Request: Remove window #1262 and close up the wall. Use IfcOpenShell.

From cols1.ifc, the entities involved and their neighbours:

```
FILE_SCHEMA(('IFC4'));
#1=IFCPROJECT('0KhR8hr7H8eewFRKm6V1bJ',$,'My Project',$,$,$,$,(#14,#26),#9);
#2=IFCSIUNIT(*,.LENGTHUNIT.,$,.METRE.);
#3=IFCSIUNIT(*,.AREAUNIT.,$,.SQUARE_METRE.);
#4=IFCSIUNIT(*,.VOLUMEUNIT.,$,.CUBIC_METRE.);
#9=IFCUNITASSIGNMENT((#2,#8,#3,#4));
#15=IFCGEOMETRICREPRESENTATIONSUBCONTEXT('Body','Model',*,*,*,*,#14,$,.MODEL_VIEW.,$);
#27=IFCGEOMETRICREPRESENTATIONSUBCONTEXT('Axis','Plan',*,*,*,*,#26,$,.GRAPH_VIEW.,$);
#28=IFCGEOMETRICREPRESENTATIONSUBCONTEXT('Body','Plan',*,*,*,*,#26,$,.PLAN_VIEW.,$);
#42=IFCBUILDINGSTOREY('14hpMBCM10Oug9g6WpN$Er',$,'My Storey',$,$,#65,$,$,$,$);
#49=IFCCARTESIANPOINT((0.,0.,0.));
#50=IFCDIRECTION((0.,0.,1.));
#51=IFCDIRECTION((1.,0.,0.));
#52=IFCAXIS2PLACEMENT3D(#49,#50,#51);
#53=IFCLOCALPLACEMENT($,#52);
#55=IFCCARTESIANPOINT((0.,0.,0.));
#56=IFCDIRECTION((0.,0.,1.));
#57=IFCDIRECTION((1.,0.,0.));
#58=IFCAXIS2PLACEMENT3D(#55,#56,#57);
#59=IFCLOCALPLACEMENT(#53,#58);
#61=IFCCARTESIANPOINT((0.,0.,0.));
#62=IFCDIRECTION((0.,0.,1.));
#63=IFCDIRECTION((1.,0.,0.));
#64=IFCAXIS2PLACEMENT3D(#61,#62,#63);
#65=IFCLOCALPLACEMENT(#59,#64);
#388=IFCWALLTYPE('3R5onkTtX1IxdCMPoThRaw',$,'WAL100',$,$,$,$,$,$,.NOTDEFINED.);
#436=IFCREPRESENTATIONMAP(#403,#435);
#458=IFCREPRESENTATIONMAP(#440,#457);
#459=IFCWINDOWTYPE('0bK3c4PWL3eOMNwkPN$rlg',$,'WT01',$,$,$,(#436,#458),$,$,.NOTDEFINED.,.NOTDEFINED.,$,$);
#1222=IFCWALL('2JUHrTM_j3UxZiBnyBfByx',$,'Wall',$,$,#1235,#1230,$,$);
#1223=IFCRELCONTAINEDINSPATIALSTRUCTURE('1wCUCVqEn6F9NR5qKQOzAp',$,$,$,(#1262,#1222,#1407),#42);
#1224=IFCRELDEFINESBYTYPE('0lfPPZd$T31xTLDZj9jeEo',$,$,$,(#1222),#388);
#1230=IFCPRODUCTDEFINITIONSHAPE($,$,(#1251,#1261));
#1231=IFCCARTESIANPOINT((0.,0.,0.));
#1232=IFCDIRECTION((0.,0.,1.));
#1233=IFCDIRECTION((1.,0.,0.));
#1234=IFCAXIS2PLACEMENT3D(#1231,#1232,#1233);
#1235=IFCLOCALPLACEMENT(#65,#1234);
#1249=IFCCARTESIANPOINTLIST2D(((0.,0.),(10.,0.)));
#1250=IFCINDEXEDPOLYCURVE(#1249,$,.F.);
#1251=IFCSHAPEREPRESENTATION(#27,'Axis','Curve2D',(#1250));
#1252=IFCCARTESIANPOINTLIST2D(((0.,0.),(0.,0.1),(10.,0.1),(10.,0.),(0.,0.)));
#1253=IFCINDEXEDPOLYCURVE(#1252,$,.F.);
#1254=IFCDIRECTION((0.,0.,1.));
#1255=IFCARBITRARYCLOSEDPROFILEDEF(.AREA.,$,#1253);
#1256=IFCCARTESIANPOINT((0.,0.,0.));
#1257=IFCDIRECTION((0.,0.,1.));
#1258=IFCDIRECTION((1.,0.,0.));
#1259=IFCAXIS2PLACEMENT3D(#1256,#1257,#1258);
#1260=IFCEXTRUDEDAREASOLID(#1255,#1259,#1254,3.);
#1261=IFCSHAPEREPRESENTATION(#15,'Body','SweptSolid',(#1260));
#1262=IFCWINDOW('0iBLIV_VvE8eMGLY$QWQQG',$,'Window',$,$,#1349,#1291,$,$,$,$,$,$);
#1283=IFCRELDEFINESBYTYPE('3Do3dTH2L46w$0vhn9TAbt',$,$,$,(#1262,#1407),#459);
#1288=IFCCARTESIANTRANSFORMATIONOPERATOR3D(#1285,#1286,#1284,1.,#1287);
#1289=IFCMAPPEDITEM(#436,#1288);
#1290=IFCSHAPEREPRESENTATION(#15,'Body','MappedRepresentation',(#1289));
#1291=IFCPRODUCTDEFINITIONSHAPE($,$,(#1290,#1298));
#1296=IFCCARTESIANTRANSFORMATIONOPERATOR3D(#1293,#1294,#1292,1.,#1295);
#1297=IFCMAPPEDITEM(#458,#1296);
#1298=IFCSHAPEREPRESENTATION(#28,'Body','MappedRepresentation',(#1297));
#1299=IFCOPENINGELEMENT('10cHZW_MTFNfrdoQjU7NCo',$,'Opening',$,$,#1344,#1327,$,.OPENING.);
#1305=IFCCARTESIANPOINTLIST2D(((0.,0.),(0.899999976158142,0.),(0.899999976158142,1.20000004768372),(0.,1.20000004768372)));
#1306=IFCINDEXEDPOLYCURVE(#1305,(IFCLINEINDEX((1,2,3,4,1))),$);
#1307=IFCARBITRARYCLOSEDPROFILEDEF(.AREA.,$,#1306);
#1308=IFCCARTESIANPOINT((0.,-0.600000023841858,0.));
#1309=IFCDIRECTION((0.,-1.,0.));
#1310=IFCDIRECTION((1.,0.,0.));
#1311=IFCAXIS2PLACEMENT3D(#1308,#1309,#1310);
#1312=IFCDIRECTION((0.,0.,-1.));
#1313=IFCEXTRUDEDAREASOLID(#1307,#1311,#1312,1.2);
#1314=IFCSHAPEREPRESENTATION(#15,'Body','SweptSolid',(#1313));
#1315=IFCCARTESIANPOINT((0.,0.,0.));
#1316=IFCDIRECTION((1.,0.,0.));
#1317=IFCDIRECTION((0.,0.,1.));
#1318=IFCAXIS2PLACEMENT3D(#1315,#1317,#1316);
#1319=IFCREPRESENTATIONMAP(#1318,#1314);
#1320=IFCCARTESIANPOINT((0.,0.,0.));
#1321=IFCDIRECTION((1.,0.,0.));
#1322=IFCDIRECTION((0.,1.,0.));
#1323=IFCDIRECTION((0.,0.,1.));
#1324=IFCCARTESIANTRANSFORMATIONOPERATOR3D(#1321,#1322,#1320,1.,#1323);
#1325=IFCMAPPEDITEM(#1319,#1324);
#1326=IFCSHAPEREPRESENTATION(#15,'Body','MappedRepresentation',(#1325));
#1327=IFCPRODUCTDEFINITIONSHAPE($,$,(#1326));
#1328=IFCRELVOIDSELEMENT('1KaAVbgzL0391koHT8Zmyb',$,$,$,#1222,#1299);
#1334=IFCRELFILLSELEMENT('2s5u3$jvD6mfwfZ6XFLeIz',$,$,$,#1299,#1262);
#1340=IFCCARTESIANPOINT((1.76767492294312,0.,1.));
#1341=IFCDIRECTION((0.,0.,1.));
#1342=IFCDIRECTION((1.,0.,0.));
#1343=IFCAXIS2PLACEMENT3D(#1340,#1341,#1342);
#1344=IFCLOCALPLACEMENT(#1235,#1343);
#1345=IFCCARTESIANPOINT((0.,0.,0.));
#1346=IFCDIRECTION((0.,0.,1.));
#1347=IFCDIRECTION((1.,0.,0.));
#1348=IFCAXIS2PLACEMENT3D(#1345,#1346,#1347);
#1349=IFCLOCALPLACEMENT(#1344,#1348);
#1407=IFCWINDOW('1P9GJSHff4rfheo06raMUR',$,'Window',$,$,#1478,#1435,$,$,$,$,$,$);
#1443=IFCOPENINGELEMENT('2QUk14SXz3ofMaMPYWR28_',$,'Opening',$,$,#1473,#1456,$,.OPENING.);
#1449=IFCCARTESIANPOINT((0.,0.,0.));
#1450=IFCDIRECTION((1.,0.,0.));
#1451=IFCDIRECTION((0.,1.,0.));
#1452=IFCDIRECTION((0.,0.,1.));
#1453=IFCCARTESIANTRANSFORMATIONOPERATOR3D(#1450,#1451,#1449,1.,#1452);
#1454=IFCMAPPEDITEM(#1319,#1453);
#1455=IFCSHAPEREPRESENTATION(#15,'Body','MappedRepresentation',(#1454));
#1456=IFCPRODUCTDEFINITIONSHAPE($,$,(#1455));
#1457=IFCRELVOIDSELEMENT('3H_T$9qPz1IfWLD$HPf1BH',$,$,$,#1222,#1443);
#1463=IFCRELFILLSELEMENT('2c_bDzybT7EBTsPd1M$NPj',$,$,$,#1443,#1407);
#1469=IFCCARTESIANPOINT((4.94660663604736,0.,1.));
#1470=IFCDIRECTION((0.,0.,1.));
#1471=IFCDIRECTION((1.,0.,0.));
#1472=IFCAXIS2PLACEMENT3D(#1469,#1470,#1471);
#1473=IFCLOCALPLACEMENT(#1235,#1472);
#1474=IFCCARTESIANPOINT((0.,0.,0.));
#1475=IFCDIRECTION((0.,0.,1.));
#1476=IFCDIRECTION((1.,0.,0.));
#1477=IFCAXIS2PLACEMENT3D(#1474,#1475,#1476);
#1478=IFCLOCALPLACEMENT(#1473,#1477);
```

```python
import ifcopenshell
import ifcopenshell.api.feature
import ifcopenshell.api.root
import ifcopenshell.geom
import ifcopenshell.util.shape

model = ifcopenshell.open("cols1.ifc")
settings = ifcopenshell.geom.settings()


def volume(element):
    """Net volume in cubic metres, openings subtracted."""
    shape = ifcopenshell.geom.create_shape(settings, element)
    return ifcopenshell.util.shape.get_volume(shape.geometry)


window = model.by_guid("0iBLIV_VvE8eMGLY$QWQQG")
opening = window.FillsVoids[0].RelatingOpeningElement
wall = opening.VoidsElements[0].RelatingBuildingElement
before = volume(wall)

ifcopenshell.api.root.remove_product(model, product=window)
ifcopenshell.api.feature.remove_feature(model, feature=opening)

after = volume(wall)

print(f"wall volume {before:.3f} -> {after:.3f} m3")

model.write("cols1-out.ifc")
```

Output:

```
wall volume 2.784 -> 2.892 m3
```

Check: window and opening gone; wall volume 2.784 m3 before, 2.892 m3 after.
